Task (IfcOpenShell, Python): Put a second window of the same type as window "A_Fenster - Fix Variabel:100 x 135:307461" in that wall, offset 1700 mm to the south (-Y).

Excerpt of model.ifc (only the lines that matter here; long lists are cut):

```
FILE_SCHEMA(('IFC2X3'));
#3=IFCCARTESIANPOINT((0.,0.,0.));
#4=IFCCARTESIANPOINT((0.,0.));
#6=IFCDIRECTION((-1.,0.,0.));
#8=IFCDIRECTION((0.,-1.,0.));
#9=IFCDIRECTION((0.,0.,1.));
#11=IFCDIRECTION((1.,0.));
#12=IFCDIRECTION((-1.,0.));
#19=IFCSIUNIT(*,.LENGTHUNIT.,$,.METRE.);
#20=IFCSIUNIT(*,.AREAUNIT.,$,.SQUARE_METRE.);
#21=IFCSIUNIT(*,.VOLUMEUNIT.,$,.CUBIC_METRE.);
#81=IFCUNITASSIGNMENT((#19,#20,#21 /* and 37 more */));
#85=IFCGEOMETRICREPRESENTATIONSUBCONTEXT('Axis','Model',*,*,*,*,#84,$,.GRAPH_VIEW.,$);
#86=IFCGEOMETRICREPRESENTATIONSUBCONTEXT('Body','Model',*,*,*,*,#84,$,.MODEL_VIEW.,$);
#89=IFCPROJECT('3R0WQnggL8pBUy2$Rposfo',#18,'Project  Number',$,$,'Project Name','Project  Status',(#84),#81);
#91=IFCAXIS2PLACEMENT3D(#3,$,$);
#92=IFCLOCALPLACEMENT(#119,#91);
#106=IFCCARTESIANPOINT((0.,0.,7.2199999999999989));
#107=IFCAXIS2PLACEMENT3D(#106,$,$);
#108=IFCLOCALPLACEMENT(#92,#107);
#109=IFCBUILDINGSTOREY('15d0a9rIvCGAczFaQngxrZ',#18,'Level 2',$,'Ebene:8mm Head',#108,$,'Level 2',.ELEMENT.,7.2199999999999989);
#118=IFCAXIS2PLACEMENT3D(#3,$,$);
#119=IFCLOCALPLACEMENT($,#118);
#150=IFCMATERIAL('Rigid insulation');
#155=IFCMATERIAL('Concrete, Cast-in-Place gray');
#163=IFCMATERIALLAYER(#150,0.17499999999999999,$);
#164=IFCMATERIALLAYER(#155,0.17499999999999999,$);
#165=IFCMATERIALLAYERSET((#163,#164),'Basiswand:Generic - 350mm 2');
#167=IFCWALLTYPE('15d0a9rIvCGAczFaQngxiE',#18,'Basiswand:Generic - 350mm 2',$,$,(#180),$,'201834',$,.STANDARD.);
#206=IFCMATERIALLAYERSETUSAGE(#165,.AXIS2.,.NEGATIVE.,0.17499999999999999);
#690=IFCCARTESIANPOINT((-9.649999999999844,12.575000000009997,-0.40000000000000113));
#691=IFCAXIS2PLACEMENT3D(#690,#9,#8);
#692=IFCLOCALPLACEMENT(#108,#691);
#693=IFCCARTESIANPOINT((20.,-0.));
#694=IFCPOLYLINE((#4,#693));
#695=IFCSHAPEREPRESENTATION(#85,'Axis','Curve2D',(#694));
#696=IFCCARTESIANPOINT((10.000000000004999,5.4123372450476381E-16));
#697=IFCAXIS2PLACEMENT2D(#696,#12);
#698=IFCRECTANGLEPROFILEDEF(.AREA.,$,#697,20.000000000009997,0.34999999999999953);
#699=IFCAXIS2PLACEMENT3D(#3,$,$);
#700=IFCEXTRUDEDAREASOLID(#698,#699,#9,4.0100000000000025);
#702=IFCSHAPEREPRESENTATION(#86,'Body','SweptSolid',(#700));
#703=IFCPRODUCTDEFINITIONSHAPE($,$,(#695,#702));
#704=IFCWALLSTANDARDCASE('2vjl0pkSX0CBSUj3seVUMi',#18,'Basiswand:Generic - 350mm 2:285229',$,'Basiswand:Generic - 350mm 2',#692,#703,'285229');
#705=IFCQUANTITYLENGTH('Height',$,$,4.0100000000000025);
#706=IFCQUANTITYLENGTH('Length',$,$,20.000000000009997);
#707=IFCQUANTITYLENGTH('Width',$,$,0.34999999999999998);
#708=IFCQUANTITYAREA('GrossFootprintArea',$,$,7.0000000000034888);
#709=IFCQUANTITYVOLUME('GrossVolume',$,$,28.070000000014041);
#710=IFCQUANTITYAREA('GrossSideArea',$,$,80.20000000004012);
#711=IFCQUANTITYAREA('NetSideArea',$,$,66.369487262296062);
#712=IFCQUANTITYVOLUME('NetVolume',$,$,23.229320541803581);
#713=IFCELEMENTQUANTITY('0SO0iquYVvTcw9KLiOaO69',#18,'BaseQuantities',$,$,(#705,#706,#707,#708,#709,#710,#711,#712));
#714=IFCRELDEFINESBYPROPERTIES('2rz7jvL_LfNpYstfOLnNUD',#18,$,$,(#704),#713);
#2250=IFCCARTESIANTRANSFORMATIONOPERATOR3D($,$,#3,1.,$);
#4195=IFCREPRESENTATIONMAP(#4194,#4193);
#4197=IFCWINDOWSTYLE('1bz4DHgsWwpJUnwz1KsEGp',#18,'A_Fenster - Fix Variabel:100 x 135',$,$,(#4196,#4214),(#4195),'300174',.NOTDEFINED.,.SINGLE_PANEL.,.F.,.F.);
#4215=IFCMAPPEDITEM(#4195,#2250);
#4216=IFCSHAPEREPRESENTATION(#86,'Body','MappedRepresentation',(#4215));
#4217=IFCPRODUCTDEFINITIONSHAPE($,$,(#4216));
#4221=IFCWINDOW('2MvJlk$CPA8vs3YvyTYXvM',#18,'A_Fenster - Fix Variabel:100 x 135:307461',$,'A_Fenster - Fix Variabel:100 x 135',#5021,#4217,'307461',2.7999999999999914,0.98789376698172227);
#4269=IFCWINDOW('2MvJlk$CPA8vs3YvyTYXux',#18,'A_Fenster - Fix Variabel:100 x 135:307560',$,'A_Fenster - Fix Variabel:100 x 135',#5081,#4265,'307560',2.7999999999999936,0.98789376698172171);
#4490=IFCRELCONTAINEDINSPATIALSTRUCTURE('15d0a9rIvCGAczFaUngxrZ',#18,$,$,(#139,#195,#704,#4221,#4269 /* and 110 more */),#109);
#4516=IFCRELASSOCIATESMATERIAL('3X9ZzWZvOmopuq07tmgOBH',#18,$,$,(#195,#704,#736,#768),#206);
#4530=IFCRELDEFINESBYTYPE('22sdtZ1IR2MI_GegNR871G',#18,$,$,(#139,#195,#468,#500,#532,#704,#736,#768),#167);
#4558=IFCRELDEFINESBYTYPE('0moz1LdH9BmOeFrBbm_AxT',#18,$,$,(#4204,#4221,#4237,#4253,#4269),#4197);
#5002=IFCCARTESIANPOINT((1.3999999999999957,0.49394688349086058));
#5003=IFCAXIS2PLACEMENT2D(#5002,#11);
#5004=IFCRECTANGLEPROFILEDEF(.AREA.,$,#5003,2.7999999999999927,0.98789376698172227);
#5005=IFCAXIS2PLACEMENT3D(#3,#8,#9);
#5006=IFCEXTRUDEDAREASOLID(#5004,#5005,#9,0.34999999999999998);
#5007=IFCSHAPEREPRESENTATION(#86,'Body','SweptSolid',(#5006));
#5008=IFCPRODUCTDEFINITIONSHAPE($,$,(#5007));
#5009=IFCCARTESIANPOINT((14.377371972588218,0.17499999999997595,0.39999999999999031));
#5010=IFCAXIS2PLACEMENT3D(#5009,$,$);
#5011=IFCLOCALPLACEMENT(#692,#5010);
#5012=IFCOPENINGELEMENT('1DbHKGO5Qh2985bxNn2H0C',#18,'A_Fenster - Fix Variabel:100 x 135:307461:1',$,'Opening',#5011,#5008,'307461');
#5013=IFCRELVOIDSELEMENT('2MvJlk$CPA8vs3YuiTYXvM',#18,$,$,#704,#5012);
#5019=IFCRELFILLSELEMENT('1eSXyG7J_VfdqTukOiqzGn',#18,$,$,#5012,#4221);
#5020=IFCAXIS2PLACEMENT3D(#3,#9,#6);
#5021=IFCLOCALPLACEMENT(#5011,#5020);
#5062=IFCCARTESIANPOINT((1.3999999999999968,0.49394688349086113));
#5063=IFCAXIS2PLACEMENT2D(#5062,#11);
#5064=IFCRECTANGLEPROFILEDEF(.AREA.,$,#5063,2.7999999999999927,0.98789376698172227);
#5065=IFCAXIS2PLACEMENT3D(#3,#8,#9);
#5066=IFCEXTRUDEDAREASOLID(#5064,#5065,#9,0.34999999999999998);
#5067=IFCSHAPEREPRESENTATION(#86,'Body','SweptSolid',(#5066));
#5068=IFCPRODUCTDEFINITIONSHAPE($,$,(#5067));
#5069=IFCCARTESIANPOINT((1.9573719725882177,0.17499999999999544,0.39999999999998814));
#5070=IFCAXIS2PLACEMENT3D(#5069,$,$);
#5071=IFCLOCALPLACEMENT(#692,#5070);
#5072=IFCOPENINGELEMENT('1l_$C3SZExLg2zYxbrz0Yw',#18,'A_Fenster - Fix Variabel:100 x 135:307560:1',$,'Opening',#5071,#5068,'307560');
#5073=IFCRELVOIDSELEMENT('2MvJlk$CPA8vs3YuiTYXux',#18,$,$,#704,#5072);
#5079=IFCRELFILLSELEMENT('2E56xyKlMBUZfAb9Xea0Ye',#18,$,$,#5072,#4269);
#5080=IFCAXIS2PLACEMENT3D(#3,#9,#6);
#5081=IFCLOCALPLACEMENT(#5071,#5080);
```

```python
import ifcopenshell
import ifcopenshell.api.feature
import ifcopenshell.api.geometry
import ifcopenshell.api.pset
import ifcopenshell.api.root
import ifcopenshell.geom
import ifcopenshell.util.element
import ifcopenshell.util.placement
import ifcopenshell.util.shape
import ifcopenshell.util.unit

model = ifcopenshell.open("model.ifc")
area_scale = ifcopenshell.util.unit.calculate_unit_scale(model, "AREAUNIT")
volume_scale = ifcopenshell.util.unit.calculate_unit_scale(model, "VOLUMEUNIT")
settings = ifcopenshell.geom.settings()


def volume(element):
    """Net volume in cubic metres, openings subtracted."""
    shape = ifcopenshell.geom.create_shape(settings, element)
    return ifcopenshell.util.shape.get_volume(shape.geometry)


def reuse_history(source, copy):
    """copy_class also copies each property set's owner history, people and application; keep the originals."""
    for rel in copy.IsDefinedBy:
        if rel.is_a("IfcRelDefinesByProperties") and (history := rel.RelatingPropertyDefinition.OwnerHistory):
            rel.RelatingPropertyDefinition.OwnerHistory = source.OwnerHistory
            ifcopenshell.util.element.remove_deep2(model, history)


window = model.by_guid("2MvJlk$CPA8vs3YvyTYXvM")
opening = window.FillsVoids[0].RelatingOpeningElement
wall = opening.VoidsElements[0].RelatingBuildingElement
before = volume(wall)
shift = ifcopenshell.util.placement.get_local_placement(wall.ObjectPlacement)[:3, 0] * 1.7

# copy_class copies the void relationship, type, container and properties, but no geometry.
new_opening = ifcopenshell.api.root.copy_class(model, product=opening)
new_opening.Representation = ifcopenshell.util.element.copy_deep(
    model, opening.Representation, exclude=["IfcGeometricRepresentationContext", "IfcRepresentationMap"]
)
new_opening.Name = "A_Fenster - Fix Variabel:100 x 135"
new_opening.Tag = None
reuse_history(opening, new_opening)
new_window = ifcopenshell.api.root.copy_class(model, product=window)
new_window.Representation = ifcopenshell.util.element.copy_deep(
    model, window.Representation, exclude=["IfcGeometricRepresentationContext", "IfcRepresentationMap"]
)
new_window.Name = "A_Fenster - Fix Variabel:100 x 135"
new_window.Tag = None
reuse_history(window, new_window)
fills = ifcopenshell.api.feature.add_filling(model, opening=new_opening, element=new_window)
fills.OwnerHistory = new_window.OwnerHistory  # required in IFC2X3

for old, new in ((opening, new_opening), (window, new_window)):
    matrix = ifcopenshell.util.placement.get_local_placement(old.ObjectPlacement)
    matrix[:3, 3] += shift
    ifcopenshell.api.geometry.edit_object_placement(model, product=new, matrix=matrix, is_si=False)

after = volume(wall)
thickness = 0.35  # wall thickness in metres

# Update the wall's stored quantities.
qto = model.by_id(ifcopenshell.util.element.get_pset(wall, "BaseQuantities", should_inherit=False)["id"])
ifcopenshell.api.pset.edit_qto(model, qto=qto, properties={
    "NetSideArea": after / thickness / area_scale,
    "NetVolume": after / volume_scale,
})

print(f"wall volume {before:.3f} -> {after:.3f} m3")

model.write("model_updated.ifc")
```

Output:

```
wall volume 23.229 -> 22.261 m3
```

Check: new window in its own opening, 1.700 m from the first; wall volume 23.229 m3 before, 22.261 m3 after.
